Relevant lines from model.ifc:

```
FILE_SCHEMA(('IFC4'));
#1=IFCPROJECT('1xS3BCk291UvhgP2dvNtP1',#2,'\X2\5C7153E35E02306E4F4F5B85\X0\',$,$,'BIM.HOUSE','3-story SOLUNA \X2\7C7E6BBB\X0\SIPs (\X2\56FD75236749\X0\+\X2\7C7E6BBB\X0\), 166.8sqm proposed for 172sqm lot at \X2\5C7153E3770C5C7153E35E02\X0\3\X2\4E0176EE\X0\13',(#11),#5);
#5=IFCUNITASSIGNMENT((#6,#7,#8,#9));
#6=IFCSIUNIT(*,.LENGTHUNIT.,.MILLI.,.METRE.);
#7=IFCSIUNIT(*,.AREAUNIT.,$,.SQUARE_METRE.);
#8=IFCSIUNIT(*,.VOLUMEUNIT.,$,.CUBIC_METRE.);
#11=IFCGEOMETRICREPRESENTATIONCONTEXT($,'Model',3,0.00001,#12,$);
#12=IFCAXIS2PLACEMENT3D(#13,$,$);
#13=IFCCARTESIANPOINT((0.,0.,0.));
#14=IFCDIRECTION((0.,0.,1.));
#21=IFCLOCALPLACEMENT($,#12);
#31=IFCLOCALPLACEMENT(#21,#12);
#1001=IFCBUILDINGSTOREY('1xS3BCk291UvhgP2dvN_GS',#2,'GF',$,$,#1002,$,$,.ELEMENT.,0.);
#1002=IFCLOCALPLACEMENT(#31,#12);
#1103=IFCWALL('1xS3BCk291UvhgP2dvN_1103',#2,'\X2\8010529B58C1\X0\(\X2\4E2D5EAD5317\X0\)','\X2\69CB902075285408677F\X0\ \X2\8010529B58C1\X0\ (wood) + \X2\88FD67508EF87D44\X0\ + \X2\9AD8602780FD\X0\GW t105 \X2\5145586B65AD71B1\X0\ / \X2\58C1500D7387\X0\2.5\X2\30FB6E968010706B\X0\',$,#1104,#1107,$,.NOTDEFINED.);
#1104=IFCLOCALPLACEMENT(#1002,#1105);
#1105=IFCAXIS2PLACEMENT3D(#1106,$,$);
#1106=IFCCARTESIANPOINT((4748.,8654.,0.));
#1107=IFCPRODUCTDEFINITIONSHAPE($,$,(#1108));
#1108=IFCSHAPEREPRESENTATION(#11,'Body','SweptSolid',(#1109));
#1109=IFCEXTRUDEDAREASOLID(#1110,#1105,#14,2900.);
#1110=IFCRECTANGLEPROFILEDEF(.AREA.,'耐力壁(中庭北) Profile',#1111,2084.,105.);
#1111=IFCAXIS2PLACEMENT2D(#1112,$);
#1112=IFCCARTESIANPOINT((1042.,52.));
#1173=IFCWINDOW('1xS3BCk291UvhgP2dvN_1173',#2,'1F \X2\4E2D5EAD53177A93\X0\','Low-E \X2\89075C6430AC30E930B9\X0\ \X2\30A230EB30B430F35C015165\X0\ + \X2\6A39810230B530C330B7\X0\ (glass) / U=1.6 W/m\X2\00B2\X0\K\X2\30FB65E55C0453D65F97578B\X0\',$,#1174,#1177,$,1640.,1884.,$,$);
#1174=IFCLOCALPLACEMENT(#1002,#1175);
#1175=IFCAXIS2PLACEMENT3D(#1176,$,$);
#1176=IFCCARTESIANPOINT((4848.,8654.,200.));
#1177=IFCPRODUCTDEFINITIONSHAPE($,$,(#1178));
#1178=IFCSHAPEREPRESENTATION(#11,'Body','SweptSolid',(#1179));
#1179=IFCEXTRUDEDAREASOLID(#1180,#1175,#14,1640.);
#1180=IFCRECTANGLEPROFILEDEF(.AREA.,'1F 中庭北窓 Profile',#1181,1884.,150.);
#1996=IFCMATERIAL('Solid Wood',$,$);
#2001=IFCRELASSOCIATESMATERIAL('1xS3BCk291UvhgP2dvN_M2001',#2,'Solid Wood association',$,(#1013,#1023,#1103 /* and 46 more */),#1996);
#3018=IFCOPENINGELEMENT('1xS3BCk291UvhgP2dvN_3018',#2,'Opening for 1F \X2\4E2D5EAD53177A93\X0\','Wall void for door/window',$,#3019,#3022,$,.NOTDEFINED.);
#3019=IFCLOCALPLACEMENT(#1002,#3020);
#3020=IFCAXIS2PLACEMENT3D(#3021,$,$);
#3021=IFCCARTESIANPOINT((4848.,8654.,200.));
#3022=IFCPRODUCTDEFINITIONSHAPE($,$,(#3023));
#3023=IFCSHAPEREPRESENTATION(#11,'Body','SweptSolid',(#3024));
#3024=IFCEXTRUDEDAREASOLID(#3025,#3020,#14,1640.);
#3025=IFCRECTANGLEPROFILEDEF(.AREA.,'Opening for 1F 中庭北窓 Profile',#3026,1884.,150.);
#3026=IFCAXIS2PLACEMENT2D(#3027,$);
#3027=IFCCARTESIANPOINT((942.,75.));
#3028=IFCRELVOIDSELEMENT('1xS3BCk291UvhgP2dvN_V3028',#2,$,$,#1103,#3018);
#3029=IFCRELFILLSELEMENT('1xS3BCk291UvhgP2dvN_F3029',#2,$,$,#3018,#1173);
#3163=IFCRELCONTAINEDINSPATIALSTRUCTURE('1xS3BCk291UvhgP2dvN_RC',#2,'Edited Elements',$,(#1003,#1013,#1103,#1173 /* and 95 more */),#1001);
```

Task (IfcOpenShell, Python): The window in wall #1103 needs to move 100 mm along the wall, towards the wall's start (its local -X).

```python
import ifcopenshell
import ifcopenshell.api.geometry
import ifcopenshell.util.placement

model = ifcopenshell.open("model.ifc")

window = model.by_guid("1xS3BCk291UvhgP2dvN_1173")
opening = window.FillsVoids[0].RelatingOpeningElement
wall = opening.VoidsElements[0].RelatingBuildingElement

wall_matrix = ifcopenshell.util.placement.get_local_placement(wall.ObjectPlacement)
shift = wall_matrix[:3, 0] * -100.0
before = ifcopenshell.util.placement.get_local_placement(window.ObjectPlacement)[:3, 3].copy()

# The window is not placed relative to its opening, so move both.
for product in (opening, window):
    matrix = ifcopenshell.util.placement.get_local_placement(product.ObjectPlacement)
    matrix[:3, 3] += shift
    ifcopenshell.api.geometry.edit_object_placement(model, product=product, matrix=matrix, is_si=False)

after = ifcopenshell.util.placement.get_local_placement(window.ObjectPlacement)[:3, 3]
print("window moved by", (after - before).round(3) + 0.0)

model.write("model_updated.ifc")
```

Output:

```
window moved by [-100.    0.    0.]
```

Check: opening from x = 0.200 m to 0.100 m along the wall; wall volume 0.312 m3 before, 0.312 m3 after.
